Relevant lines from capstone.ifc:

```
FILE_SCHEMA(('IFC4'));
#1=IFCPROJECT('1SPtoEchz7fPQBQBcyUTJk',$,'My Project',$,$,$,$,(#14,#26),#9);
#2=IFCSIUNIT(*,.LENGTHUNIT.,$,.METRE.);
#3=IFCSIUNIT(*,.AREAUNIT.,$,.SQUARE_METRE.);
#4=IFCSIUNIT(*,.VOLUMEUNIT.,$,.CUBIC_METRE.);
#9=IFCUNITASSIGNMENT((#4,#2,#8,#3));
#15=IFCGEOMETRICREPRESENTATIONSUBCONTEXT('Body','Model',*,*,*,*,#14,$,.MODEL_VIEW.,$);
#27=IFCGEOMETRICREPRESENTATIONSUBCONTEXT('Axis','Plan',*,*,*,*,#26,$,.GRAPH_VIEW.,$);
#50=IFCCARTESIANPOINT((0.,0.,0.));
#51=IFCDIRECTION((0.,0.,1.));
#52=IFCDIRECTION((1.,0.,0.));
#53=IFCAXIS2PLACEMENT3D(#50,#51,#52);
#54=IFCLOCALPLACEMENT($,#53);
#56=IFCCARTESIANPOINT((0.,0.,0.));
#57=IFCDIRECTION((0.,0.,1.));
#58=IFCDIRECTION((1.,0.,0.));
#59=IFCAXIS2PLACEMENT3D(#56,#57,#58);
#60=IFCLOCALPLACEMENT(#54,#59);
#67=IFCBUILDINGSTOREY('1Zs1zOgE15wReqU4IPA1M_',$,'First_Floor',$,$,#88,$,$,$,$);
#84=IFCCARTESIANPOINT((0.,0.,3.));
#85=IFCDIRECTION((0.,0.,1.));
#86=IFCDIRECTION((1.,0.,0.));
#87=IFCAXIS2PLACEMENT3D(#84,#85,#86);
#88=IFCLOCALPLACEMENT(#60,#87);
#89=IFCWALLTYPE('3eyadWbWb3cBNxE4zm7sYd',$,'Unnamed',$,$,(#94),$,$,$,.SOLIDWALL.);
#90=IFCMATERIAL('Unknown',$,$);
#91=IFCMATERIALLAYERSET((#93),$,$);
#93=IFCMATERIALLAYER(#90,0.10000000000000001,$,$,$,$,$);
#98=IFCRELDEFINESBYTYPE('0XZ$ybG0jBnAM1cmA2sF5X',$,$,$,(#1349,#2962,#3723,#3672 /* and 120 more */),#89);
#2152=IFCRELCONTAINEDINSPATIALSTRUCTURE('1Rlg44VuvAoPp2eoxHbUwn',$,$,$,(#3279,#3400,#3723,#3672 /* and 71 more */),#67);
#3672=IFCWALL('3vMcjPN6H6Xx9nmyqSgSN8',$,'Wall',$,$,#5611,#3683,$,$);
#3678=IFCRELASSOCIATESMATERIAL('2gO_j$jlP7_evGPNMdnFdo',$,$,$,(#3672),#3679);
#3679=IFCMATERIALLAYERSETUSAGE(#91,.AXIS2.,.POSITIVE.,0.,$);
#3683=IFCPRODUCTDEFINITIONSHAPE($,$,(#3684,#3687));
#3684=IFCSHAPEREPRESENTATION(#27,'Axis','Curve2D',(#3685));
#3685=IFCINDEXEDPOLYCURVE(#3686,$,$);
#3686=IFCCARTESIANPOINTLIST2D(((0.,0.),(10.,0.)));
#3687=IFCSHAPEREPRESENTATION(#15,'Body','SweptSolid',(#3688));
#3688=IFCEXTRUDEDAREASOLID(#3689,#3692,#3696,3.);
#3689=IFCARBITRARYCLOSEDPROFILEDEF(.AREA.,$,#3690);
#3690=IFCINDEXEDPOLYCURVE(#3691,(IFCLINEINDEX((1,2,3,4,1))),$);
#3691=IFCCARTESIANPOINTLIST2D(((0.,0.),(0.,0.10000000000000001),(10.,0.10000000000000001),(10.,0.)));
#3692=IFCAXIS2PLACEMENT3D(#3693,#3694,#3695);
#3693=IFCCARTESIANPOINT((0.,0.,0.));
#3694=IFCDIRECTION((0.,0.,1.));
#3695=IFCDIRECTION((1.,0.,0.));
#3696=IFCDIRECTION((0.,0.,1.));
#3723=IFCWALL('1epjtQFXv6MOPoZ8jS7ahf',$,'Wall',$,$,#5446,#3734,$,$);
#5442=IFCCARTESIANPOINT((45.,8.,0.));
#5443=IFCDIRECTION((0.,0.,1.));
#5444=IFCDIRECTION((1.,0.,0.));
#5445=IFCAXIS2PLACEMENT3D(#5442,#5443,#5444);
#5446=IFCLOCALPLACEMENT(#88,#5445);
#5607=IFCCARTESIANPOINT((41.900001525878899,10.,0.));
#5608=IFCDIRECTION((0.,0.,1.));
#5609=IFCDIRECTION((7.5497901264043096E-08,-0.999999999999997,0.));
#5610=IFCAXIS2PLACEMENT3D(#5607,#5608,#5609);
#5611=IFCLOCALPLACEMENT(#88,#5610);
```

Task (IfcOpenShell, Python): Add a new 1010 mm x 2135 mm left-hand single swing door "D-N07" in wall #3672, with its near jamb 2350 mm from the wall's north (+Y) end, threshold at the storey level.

```python
import numpy as np
import ifcopenshell
import ifcopenshell.api.feature
import ifcopenshell.api.geometry
import ifcopenshell.api.root
import ifcopenshell.api.spatial
import ifcopenshell.geom
import ifcopenshell.util.element
import ifcopenshell.util.placement
import ifcopenshell.util.representation
import ifcopenshell.util.shape
import ifcopenshell.util.unit

model = ifcopenshell.open("capstone.ifc")
unit_scale = ifcopenshell.util.unit.calculate_unit_scale(model)
settings = ifcopenshell.geom.settings()


def volume(element):
    """Net volume in cubic metres, openings subtracted."""
    shape = ifcopenshell.geom.create_shape(settings, element)
    return ifcopenshell.util.shape.get_volume(shape.geometry)


wall = model.by_guid("3vMcjPN6H6Xx9nmyqSgSN8")
storey = ifcopenshell.util.element.get_container(wall, ifc_class="IfcBuildingStorey")
context = ifcopenshell.util.representation.get_context(model, "Model", "Body", "MODEL_VIEW")
before = volume(wall)

width, height, from_end, sill = 1.01, 2.135, 2.35, 0.0  # metres

# The wall runs along its own X axis, and the end named is its -X end.
wall_shape = ifcopenshell.geom.create_shape(settings, wall)
x, y, z = ifcopenshell.util.shape.get_vertices(wall_shape.geometry).T
start = x.min() + from_end
face, thickness = float(y.min()), float(y.max() - y.min())
wall_matrix = ifcopenshell.util.placement.get_local_placement(wall.ObjectPlacement)
level = ifcopenshell.util.placement.get_local_placement(storey.ObjectPlacement)[2, 3]


def in_wall(x, y):
    """Placement at x, y metres in the wall's axes, at sill height."""
    matrix = wall_matrix.copy()
    matrix[:, 3] = wall_matrix @ np.array([x / unit_scale, y / unit_scale, 0.0, 1.0])
    matrix[2, 3] = level + sill / unit_scale
    return matrix


# Opening: a box that overshoots both wall faces by 50 mm.
opening = ifcopenshell.api.root.create_entity(model, ifc_class="IfcOpeningElement", predefined_type="OPENING")
box = ifcopenshell.api.geometry.add_wall_representation(
    model, context=context, length=width, height=height, thickness=thickness + 0.1
)
ifcopenshell.api.geometry.assign_representation(model, product=opening, representation=box)
ifcopenshell.api.geometry.edit_object_placement(model, product=opening, matrix=in_wall(start, face - 0.05), is_si=False)
ifcopenshell.api.feature.add_feature(model, feature=opening, element=wall)

door = ifcopenshell.api.root.create_entity(model, ifc_class="IfcDoor", name="D-N07", predefined_type="DOOR")
door.OverallWidth, door.OverallHeight = width / unit_scale, height / unit_scale
door.OperationType = "SINGLE_SWING_LEFT"
body = ifcopenshell.api.geometry.add_door_representation(
    model,
    context=context,
    overall_width=door.OverallWidth,
    overall_height=door.OverallHeight,
    operation_type="SINGLE_SWING_LEFT",
    lining_properties={"LiningDepth": thickness / unit_scale, "ThresholdDepth": thickness / unit_scale},
)
ifcopenshell.api.geometry.assign_representation(model, product=door, representation=body)
ifcopenshell.api.spatial.assign_container(model, products=[door], relating_structure=storey)
ifcopenshell.api.feature.add_filling(model, opening=opening, element=door)

# The lining spans the wall, so the door starts at the wall face.
ifcopenshell.api.geometry.edit_object_placement(model, product=door, matrix=in_wall(start, face), is_si=False)

after = volume(wall)

print(f"wall volume {before:.3f} -> {after:.3f} m3")

model.write("capstone_v2.ifc")
```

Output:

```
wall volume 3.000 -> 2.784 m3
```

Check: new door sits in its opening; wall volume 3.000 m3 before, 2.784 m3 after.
